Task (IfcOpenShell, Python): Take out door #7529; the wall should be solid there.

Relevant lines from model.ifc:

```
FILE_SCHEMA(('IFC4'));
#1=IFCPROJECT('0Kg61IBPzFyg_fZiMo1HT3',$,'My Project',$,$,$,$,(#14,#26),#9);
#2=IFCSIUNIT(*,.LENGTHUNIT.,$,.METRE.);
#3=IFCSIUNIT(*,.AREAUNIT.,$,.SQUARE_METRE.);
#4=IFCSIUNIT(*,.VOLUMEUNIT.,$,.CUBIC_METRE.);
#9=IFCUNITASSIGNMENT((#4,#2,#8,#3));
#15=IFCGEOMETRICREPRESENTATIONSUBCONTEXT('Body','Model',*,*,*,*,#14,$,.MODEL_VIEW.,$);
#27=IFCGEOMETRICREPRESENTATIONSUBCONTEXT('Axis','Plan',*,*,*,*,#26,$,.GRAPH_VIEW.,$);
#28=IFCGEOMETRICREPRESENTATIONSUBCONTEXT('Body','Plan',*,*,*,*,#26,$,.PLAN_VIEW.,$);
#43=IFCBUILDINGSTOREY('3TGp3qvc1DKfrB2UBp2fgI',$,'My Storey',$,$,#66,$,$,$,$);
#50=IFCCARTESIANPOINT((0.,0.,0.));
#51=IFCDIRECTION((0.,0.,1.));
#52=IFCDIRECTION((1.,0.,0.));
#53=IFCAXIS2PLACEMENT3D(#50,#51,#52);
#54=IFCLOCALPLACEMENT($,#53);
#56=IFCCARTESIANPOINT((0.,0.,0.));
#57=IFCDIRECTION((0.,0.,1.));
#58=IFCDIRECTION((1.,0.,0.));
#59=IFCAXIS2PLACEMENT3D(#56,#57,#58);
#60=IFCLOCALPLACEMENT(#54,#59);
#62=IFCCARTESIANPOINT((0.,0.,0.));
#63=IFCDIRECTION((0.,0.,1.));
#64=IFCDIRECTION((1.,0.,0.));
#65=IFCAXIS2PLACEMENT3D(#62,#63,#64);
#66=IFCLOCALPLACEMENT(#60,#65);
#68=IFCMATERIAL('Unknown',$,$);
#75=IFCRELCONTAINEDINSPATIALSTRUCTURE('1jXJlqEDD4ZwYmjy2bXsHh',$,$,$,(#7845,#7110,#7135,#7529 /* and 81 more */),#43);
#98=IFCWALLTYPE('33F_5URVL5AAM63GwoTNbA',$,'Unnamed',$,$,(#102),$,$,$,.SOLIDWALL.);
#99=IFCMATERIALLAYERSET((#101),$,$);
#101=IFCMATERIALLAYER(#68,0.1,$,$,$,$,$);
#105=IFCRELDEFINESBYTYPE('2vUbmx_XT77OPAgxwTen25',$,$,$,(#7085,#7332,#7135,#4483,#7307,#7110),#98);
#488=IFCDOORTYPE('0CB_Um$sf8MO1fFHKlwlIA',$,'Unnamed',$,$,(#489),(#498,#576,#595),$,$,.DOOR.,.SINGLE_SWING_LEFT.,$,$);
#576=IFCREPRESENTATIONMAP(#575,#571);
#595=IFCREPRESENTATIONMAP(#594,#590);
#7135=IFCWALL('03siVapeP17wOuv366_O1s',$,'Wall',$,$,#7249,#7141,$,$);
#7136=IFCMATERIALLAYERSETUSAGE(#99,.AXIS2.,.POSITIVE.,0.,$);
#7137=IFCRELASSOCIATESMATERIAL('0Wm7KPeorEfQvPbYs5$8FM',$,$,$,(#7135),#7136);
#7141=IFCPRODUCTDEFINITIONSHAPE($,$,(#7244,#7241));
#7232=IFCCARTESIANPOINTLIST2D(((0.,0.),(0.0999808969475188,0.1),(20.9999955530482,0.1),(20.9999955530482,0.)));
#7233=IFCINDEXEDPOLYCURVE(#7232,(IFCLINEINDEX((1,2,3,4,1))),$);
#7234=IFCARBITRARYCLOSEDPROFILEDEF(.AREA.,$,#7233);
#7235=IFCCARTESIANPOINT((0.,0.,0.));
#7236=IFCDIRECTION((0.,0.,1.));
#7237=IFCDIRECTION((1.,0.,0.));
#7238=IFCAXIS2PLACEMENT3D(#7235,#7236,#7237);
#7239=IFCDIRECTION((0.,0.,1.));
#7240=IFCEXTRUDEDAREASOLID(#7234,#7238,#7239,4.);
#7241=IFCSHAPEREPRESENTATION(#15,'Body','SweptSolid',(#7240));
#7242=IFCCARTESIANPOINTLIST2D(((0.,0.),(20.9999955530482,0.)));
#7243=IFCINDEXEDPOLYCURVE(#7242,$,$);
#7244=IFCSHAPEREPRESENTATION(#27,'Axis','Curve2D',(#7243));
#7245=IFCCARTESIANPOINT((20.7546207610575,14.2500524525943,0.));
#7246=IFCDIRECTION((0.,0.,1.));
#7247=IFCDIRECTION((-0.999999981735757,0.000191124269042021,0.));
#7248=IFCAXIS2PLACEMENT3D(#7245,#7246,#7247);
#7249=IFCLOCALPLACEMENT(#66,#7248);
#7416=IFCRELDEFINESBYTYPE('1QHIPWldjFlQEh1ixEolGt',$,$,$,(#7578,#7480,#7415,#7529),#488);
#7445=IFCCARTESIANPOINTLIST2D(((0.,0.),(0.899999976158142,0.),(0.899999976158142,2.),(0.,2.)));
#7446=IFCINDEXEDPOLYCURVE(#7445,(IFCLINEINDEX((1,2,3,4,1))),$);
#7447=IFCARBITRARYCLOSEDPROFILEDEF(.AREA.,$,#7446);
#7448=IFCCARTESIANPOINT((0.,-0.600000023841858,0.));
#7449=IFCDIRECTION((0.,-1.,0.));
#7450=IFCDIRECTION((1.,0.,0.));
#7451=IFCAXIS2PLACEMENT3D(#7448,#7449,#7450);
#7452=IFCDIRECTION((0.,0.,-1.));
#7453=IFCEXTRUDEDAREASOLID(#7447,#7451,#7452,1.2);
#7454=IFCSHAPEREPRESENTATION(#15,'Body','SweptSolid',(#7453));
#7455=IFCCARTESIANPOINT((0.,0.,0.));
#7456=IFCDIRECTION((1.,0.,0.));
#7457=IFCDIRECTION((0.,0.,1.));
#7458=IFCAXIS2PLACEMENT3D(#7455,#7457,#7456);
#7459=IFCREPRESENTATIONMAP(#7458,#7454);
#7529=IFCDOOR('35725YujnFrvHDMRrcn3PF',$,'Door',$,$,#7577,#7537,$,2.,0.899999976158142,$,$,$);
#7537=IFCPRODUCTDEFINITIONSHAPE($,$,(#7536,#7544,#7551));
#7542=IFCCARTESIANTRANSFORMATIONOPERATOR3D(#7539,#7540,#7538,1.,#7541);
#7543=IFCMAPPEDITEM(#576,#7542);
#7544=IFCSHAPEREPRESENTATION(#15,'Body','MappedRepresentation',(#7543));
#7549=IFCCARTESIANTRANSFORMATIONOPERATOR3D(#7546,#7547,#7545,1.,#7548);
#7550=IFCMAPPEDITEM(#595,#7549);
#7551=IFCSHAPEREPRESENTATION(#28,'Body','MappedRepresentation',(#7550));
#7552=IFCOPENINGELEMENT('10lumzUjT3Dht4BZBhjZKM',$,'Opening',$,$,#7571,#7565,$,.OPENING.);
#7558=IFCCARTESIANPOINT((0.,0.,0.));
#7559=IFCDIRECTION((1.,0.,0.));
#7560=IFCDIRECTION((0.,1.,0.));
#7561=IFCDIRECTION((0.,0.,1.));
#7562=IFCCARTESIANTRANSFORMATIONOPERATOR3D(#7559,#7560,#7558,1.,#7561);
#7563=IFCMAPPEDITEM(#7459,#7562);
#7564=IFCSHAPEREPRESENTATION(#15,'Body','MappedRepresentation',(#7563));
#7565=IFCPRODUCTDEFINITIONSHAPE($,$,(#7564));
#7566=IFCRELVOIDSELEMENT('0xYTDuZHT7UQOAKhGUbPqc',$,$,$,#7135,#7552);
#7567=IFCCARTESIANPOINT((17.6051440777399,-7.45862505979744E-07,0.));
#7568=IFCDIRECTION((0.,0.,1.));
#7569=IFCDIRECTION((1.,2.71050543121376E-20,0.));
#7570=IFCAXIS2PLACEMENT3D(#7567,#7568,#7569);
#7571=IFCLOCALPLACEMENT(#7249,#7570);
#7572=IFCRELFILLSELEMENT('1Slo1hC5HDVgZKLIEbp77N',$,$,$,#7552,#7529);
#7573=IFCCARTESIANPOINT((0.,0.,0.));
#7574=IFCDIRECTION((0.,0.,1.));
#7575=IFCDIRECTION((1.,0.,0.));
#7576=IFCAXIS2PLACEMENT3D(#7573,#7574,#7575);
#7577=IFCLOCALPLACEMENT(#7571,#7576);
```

```python
import ifcopenshell
import ifcopenshell.api.feature
import ifcopenshell.api.root
import ifcopenshell.geom
import ifcopenshell.util.shape

model = ifcopenshell.open("model.ifc")
settings = ifcopenshell.geom.settings()


def volume(element):
    """Net volume in cubic metres, openings subtracted."""
    shape = ifcopenshell.geom.create_shape(settings, element)
    return ifcopenshell.util.shape.get_volume(shape.geometry)


door = model.by_id(7529)
opening = door.FillsVoids[0].RelatingOpeningElement
wall = opening.VoidsElements[0].RelatingBuildingElement
before = volume(wall)

ifcopenshell.api.root.remove_product(model, product=door)
ifcopenshell.api.feature.remove_feature(model, feature=opening)

after = volume(wall)

print(f"wall volume {before:.3f} -> {after:.3f} m3")

model.write("model_edited.ifc")
```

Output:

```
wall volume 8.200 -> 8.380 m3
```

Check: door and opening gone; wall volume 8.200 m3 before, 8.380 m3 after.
